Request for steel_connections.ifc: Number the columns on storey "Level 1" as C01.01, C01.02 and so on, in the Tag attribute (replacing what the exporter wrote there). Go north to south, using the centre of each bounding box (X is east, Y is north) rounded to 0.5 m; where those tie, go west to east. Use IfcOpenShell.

First a look at what the model holds.

```python
import ifcopenshell
import ifcopenshell.util.element
import ifcopenshell.util.placement

model = ifcopenshell.open("steel_connections.ifc")
print(model.schema)
storey = next(s for s in model.by_type("IfcBuildingStorey") if s.Name == "Level 1")
columns = [e for e in ifcopenshell.util.element.get_decomposition(storey) if e.is_a("IfcColumn")]
for e in sorted(columns, key=lambda e: e.id()):
    origin = ifcopenshell.util.placement.get_local_placement(e.ObjectPlacement)[:3, 3]
    print(e.id(), e.Tag, e.Name, origin.round(2) + 0.0, sep=" | ")
```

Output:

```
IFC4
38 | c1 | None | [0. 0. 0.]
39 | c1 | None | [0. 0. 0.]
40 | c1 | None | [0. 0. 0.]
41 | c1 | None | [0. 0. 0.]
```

```python
import ifcopenshell
import ifcopenshell.geom
import ifcopenshell.util.element
import ifcopenshell.util.shape

model = ifcopenshell.open("steel_connections.ifc")
settings = ifcopenshell.geom.settings()
settings.set("use-world-coords", True)


def centre(element):
    shape = ifcopenshell.geom.create_shape(settings, element)
    return ifcopenshell.util.shape.get_bbox_centroid(shape.geometry)


storey = next(s for s in model.by_type("IfcBuildingStorey") if s.Name == "Level 1")
columns = [e for e in ifcopenshell.util.element.get_decomposition(storey) if e.is_a("IfcColumn")]

# Insertion points can sit at a corner or the storey origin, so sort by the geometry (in metres).
centres = {e: centre(e) for e in columns}
columns.sort(key=lambda e: (-round(centres[e][1] / 0.5), centres[e][0]))

for i, e in enumerate(columns, start=1):
    number = f"C01.{i:02d}"
    e.Tag = number
    print(e.id(), number)

model.write("steel_connections_edited.ifc")
```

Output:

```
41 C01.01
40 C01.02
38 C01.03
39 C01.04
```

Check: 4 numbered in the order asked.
